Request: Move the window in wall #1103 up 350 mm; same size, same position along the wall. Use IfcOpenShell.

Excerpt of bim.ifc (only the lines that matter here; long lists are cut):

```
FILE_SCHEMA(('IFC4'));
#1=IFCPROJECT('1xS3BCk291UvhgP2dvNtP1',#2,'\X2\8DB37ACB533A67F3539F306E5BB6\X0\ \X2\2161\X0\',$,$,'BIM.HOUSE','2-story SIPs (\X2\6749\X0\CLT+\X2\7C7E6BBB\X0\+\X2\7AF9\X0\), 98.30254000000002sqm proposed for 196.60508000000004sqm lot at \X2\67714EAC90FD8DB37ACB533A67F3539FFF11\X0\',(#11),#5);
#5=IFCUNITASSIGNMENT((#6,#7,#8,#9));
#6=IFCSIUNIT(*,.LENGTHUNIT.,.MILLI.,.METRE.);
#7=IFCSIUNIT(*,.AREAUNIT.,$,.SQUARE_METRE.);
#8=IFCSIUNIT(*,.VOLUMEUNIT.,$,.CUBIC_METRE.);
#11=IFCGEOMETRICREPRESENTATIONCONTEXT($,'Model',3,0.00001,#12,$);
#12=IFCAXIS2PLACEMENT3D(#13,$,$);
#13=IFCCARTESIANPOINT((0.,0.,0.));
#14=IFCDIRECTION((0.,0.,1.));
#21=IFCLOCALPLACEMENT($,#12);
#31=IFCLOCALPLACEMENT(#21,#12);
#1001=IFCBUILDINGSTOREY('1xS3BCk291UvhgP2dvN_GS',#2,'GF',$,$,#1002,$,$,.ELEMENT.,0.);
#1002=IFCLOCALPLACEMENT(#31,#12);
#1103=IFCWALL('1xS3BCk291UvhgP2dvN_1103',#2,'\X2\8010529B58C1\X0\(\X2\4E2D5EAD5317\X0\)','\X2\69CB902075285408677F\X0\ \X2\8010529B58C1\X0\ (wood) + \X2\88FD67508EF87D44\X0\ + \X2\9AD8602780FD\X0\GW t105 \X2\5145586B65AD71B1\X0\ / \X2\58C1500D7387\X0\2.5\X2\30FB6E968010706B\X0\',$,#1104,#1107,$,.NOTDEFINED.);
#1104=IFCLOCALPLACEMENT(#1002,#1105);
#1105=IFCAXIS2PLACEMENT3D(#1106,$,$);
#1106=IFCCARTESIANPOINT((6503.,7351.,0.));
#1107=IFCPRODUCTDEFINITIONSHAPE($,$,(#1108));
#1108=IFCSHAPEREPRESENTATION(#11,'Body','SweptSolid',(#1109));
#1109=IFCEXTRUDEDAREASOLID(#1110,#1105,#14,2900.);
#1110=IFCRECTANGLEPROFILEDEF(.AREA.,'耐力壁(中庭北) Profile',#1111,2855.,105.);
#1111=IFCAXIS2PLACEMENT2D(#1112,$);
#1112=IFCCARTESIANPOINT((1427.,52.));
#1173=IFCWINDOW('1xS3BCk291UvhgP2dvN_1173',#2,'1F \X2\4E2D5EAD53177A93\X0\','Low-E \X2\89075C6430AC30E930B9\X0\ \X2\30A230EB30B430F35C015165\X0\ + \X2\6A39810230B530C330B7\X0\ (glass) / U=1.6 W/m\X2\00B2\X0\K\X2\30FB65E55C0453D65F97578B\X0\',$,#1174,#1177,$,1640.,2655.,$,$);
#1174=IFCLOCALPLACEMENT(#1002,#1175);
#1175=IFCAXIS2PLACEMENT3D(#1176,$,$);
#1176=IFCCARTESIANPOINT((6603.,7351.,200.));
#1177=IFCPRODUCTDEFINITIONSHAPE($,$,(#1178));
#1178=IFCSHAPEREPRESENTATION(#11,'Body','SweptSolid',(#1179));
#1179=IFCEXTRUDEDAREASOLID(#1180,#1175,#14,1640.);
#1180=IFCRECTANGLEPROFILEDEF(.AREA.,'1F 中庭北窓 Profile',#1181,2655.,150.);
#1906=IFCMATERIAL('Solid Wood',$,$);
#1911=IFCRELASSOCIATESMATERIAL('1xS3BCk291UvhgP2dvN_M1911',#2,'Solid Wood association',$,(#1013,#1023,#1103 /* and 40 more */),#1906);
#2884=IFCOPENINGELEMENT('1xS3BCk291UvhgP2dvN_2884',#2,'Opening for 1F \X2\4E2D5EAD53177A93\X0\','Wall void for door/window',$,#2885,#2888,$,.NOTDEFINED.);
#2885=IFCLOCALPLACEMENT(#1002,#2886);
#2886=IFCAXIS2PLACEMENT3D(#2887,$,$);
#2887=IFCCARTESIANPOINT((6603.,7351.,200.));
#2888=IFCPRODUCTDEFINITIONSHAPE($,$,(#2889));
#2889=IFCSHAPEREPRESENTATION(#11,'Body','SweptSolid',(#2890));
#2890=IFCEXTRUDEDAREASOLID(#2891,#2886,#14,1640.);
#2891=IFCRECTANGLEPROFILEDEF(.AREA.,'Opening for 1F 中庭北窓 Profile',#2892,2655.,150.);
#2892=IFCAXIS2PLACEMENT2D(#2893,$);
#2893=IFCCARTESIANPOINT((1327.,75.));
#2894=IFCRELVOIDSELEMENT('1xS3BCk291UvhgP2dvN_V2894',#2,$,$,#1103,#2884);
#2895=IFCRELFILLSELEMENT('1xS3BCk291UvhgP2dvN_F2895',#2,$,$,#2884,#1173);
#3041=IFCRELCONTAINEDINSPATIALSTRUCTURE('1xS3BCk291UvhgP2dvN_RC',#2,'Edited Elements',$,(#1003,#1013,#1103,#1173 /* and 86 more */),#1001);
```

```python
import numpy as np
import ifcopenshell
import ifcopenshell.api.geometry
import ifcopenshell.util.placement
import ifcopenshell.util.unit

model = ifcopenshell.open("bim.ifc")
unit_scale = ifcopenshell.util.unit.calculate_unit_scale(model)

window = model.by_guid("1xS3BCk291UvhgP2dvN_1173")
opening = window.FillsVoids[0].RelatingOpeningElement
dz = 0.35 / unit_scale

shift = np.array([0.0, 0.0, dz])
# The window is not placed relative to its opening, so move both.
for product in (opening, window):
    matrix = ifcopenshell.util.placement.get_local_placement(product.ObjectPlacement)
    matrix[:3, 3] += shift
    ifcopenshell.api.geometry.edit_object_placement(model, product=product, matrix=matrix, is_si=False)

print(f"moved by {dz * unit_scale:+.3f} m")

model.write("bim_updated.ifc")
```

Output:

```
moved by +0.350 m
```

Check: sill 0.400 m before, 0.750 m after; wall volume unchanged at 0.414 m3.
